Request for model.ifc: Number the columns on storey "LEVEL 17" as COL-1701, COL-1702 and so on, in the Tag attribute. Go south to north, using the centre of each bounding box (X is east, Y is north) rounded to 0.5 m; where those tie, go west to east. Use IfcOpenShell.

First a look at what the model holds.

```python
import ifcopenshell
import ifcopenshell.util.element
import ifcopenshell.util.placement

model = ifcopenshell.open("model.ifc")
print(model.schema)
storey = next(s for s in model.by_type("IfcBuildingStorey") if s.Name == "LEVEL 17")
columns = [e for e in ifcopenshell.util.element.get_decomposition(storey) if e.is_a("IfcColumn")]
for e in sorted(columns, key=lambda e: e.id()):
    origin = ifcopenshell.util.placement.get_local_placement(e.ObjectPlacement)[:3, 3]
    print(e.id(), e.Tag, e.Name, origin.round(2) + 0.0, sep=" | ")
```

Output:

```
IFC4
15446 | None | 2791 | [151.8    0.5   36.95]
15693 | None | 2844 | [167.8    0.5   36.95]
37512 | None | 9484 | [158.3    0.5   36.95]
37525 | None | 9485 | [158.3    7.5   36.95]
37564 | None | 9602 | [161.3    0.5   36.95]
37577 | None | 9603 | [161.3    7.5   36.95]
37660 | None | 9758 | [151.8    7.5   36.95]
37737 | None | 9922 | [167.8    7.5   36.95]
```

```python
import ifcopenshell
import ifcopenshell.geom
import ifcopenshell.util.element
import ifcopenshell.util.shape

model = ifcopenshell.open("model.ifc")
settings = ifcopenshell.geom.settings()
settings.set("use-world-coords", True)


def centre(element):
    shape = ifcopenshell.geom.create_shape(settings, element)
    return ifcopenshell.util.shape.get_bbox_centroid(shape.geometry)


storey = next(s for s in model.by_type("IfcBuildingStorey") if s.Name == "LEVEL 17")
columns = [e for e in ifcopenshell.util.element.get_decomposition(storey) if e.is_a("IfcColumn")]

# Insertion points can sit at a corner or the storey origin, so sort by the geometry (in metres).
centres = {e: centre(e) for e in columns}
columns.sort(key=lambda e: (round(centres[e][1] / 0.5), centres[e][0]))

for i, e in enumerate(columns, start=1):
    number = f"COL-17{i:02d}"
    e.Tag = number
    print(e.id(), number)

model.write("model_v2.ifc")
```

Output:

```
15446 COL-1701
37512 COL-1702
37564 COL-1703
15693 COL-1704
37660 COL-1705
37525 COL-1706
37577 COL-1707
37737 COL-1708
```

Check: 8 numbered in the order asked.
